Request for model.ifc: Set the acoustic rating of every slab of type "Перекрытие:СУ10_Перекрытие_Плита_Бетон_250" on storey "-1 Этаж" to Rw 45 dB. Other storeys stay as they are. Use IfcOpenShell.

First a look at what the model holds.

```python
import ifcopenshell
import ifcopenshell.util.element

model = ifcopenshell.open("model.ifc")
print(model.schema)
storey = next(s for s in model.by_type("IfcBuildingStorey") if s.Name == "-1 Этаж")
slabs = [e for e in ifcopenshell.util.element.get_decomposition(storey) if e.is_a("IfcSlab")]
seen = {}
for e in slabs:
    element_type = ifcopenshell.util.element.get_type(e)
    key = (element_type.Name if element_type != e and element_type else None, ifcopenshell.util.element.get_pset(e, "Pset_SlabCommon", "AcousticRating"))
    seen[key] = seen.get(key, 0) + 1
for (name, value), count in sorted(seen.items(), key=str):
    print(count, "x", name, "|", value)
```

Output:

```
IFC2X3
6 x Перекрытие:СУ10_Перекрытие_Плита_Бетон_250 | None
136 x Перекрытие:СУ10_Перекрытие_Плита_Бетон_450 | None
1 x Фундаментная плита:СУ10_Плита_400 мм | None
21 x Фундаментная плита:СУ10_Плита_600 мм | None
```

```python
import ifcopenshell
import ifcopenshell.api.pset
import ifcopenshell.util.element

model = ifcopenshell.open("model.ifc")

storey = next(s for s in model.by_type("IfcBuildingStorey") if s.Name == "-1 Этаж")
slabs = [e for e in ifcopenshell.util.element.get_decomposition(storey) if e.is_a("IfcSlab")]

count = 0
for e in slabs:
    element_type = ifcopenshell.util.element.get_type(e)
    if element_type in (None, e) or element_type.Name != "Перекрытие:СУ10_Перекрытие_Плита_Бетон_250":
        continue
    # add_pset returns the element's existing set when there is one.
    pset = ifcopenshell.api.pset.add_pset(model, product=e, name="Pset_SlabCommon")
    ifcopenshell.api.pset.edit_pset(model, pset=pset, properties={"AcousticRating": "Rw 45 dB"})
    count += 1

print(count, "slabs updated")

model.write("model_updated.ifc")
```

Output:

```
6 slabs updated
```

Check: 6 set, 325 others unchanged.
